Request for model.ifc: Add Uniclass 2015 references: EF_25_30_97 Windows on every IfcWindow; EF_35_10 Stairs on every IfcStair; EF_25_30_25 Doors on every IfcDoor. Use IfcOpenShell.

First a look at what the model holds.

```python
import ifcopenshell

model = ifcopenshell.open("model.ifc")
print(model.schema)
print("classifications:", [c.Name for c in model.by_type("IfcClassification")])
for ifc_class in ("IfcDoor", "IfcRoof", "IfcStair", "IfcWall", "IfcWindow"):
    print(ifc_class, len(model.by_type(ifc_class)))
```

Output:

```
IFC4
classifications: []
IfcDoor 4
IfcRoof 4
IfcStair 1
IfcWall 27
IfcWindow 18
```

```python
import ifcopenshell
import ifcopenshell.api.classification

model = ifcopenshell.open("model.ifc")

system = ifcopenshell.api.classification.add_classification(model, classification="Uniclass 2015")

codes = {
    "IfcWindow": ("EF_25_30_97", "Windows"),
    "IfcStair": ("EF_35_10", "Stairs"),
    "IfcDoor": ("EF_25_30_25", "Doors"),
}
for ifc_class, (code, name) in codes.items():
    products = model.by_type(ifc_class)
    ifcopenshell.api.classification.add_reference(
        model, products=products, classification=system, identification=code, name=name
    )
    print(code, len(products))

model.write("model_edited.ifc")
```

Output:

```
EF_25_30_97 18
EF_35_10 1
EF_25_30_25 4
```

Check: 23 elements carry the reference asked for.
